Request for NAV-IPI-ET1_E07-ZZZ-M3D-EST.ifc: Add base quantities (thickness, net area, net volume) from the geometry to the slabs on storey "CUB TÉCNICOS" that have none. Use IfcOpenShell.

First a look at what the model holds.

```python
import ifcopenshell
import ifcopenshell.util.element
import ifcopenshell.util.unit

model = ifcopenshell.open("NAV-IPI-ET1_E07-ZZZ-M3D-EST.ifc")
print(model.schema)
for unit_type in ("LENGTHUNIT", "AREAUNIT", "VOLUMEUNIT"):
    print(unit_type, ifcopenshell.util.unit.calculate_unit_scale(model, unit_type))
storey = next(s for s in model.by_type("IfcBuildingStorey") if s.Name == "CUB TÉCNICOS")
slabs = [e for e in ifcopenshell.util.element.get_decomposition(storey) if e.is_a("IfcSlab")]
for e in sorted(slabs, key=lambda e: e.id()):
    print(e.id(), e.is_a(), e.Name, list(ifcopenshell.util.element.get_psets(e, qtos_only=True)), sep=" | ")
```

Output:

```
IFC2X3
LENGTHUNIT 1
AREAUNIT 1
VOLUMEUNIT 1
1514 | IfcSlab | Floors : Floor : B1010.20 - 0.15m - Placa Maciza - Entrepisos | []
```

```python
import ifcopenshell
import ifcopenshell.api.pset
import ifcopenshell.geom
import ifcopenshell.util.element
import ifcopenshell.util.shape
import ifcopenshell.util.unit

model = ifcopenshell.open("NAV-IPI-ET1_E07-ZZZ-M3D-EST.ifc")
unit_scale = ifcopenshell.util.unit.calculate_unit_scale(model)
area_scale = ifcopenshell.util.unit.calculate_unit_scale(model, "AREAUNIT")
volume_scale = ifcopenshell.util.unit.calculate_unit_scale(model, "VOLUMEUNIT")
settings = ifcopenshell.geom.settings()

storey = next(s for s in model.by_type("IfcBuildingStorey") if s.Name == "CUB TÉCNICOS")
slabs = [e for e in ifcopenshell.util.element.get_decomposition(storey) if e.is_a("IfcSlab")]

for e in sorted(slabs, key=lambda e: e.id()):
    if ifcopenshell.util.element.get_psets(e, qtos_only=True, should_inherit=False):
        continue
    # Geometry comes back in metres, in the element's own axes.
    shape = ifcopenshell.geom.create_shape(settings, e)
    values = {
        "Width": ifcopenshell.util.shape.get_z(shape.geometry) / unit_scale,
        "NetArea": ifcopenshell.util.shape.get_footprint_area(shape.geometry) / area_scale,
        "NetVolume": ifcopenshell.util.shape.get_volume(shape.geometry) / volume_scale,
    }
    qto = ifcopenshell.api.pset.add_qto(model, product=e, name="BaseQuantities")
    ifcopenshell.api.pset.edit_qto(model, qto=qto, properties=values)
    print(e.id(), {k: round(v, 3) for k, v in values.items()})

model.write("NAV-IPI-ET1_E07-ZZZ-M3D-EST-out.ifc")
```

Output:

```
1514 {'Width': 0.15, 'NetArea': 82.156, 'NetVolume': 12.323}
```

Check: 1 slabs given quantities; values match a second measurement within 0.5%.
